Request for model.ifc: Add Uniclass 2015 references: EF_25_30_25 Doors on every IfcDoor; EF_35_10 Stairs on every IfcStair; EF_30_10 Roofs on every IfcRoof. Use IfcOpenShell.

First a look at what the model holds.

```python
import ifcopenshell

model = ifcopenshell.open("model.ifc")
print(model.schema)
print("classifications:", [c.Name for c in model.by_type("IfcClassification")])
for ifc_class in ("IfcDoor", "IfcRoof", "IfcStair", "IfcWall", "IfcWindow"):
    print(ifc_class, len(model.by_type(ifc_class)))
```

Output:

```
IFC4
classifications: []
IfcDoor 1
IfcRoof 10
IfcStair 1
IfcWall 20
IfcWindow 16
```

```python
import ifcopenshell
import ifcopenshell.api.classification

model = ifcopenshell.open("model.ifc")

system = ifcopenshell.api.classification.add_classification(model, classification="Uniclass 2015")

codes = {
    "IfcDoor": ("EF_25_30_25", "Doors"),
    "IfcStair": ("EF_35_10", "Stairs"),
    "IfcRoof": ("EF_30_10", "Roofs"),
}
for ifc_class, (code, name) in codes.items():
    products = model.by_type(ifc_class)
    ifcopenshell.api.classification.add_reference(
        model, products=products, classification=system, identification=code, name=name
    )
    print(code, len(products))

model.write("model_rev.ifc")
```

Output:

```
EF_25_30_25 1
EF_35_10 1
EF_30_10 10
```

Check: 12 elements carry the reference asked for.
